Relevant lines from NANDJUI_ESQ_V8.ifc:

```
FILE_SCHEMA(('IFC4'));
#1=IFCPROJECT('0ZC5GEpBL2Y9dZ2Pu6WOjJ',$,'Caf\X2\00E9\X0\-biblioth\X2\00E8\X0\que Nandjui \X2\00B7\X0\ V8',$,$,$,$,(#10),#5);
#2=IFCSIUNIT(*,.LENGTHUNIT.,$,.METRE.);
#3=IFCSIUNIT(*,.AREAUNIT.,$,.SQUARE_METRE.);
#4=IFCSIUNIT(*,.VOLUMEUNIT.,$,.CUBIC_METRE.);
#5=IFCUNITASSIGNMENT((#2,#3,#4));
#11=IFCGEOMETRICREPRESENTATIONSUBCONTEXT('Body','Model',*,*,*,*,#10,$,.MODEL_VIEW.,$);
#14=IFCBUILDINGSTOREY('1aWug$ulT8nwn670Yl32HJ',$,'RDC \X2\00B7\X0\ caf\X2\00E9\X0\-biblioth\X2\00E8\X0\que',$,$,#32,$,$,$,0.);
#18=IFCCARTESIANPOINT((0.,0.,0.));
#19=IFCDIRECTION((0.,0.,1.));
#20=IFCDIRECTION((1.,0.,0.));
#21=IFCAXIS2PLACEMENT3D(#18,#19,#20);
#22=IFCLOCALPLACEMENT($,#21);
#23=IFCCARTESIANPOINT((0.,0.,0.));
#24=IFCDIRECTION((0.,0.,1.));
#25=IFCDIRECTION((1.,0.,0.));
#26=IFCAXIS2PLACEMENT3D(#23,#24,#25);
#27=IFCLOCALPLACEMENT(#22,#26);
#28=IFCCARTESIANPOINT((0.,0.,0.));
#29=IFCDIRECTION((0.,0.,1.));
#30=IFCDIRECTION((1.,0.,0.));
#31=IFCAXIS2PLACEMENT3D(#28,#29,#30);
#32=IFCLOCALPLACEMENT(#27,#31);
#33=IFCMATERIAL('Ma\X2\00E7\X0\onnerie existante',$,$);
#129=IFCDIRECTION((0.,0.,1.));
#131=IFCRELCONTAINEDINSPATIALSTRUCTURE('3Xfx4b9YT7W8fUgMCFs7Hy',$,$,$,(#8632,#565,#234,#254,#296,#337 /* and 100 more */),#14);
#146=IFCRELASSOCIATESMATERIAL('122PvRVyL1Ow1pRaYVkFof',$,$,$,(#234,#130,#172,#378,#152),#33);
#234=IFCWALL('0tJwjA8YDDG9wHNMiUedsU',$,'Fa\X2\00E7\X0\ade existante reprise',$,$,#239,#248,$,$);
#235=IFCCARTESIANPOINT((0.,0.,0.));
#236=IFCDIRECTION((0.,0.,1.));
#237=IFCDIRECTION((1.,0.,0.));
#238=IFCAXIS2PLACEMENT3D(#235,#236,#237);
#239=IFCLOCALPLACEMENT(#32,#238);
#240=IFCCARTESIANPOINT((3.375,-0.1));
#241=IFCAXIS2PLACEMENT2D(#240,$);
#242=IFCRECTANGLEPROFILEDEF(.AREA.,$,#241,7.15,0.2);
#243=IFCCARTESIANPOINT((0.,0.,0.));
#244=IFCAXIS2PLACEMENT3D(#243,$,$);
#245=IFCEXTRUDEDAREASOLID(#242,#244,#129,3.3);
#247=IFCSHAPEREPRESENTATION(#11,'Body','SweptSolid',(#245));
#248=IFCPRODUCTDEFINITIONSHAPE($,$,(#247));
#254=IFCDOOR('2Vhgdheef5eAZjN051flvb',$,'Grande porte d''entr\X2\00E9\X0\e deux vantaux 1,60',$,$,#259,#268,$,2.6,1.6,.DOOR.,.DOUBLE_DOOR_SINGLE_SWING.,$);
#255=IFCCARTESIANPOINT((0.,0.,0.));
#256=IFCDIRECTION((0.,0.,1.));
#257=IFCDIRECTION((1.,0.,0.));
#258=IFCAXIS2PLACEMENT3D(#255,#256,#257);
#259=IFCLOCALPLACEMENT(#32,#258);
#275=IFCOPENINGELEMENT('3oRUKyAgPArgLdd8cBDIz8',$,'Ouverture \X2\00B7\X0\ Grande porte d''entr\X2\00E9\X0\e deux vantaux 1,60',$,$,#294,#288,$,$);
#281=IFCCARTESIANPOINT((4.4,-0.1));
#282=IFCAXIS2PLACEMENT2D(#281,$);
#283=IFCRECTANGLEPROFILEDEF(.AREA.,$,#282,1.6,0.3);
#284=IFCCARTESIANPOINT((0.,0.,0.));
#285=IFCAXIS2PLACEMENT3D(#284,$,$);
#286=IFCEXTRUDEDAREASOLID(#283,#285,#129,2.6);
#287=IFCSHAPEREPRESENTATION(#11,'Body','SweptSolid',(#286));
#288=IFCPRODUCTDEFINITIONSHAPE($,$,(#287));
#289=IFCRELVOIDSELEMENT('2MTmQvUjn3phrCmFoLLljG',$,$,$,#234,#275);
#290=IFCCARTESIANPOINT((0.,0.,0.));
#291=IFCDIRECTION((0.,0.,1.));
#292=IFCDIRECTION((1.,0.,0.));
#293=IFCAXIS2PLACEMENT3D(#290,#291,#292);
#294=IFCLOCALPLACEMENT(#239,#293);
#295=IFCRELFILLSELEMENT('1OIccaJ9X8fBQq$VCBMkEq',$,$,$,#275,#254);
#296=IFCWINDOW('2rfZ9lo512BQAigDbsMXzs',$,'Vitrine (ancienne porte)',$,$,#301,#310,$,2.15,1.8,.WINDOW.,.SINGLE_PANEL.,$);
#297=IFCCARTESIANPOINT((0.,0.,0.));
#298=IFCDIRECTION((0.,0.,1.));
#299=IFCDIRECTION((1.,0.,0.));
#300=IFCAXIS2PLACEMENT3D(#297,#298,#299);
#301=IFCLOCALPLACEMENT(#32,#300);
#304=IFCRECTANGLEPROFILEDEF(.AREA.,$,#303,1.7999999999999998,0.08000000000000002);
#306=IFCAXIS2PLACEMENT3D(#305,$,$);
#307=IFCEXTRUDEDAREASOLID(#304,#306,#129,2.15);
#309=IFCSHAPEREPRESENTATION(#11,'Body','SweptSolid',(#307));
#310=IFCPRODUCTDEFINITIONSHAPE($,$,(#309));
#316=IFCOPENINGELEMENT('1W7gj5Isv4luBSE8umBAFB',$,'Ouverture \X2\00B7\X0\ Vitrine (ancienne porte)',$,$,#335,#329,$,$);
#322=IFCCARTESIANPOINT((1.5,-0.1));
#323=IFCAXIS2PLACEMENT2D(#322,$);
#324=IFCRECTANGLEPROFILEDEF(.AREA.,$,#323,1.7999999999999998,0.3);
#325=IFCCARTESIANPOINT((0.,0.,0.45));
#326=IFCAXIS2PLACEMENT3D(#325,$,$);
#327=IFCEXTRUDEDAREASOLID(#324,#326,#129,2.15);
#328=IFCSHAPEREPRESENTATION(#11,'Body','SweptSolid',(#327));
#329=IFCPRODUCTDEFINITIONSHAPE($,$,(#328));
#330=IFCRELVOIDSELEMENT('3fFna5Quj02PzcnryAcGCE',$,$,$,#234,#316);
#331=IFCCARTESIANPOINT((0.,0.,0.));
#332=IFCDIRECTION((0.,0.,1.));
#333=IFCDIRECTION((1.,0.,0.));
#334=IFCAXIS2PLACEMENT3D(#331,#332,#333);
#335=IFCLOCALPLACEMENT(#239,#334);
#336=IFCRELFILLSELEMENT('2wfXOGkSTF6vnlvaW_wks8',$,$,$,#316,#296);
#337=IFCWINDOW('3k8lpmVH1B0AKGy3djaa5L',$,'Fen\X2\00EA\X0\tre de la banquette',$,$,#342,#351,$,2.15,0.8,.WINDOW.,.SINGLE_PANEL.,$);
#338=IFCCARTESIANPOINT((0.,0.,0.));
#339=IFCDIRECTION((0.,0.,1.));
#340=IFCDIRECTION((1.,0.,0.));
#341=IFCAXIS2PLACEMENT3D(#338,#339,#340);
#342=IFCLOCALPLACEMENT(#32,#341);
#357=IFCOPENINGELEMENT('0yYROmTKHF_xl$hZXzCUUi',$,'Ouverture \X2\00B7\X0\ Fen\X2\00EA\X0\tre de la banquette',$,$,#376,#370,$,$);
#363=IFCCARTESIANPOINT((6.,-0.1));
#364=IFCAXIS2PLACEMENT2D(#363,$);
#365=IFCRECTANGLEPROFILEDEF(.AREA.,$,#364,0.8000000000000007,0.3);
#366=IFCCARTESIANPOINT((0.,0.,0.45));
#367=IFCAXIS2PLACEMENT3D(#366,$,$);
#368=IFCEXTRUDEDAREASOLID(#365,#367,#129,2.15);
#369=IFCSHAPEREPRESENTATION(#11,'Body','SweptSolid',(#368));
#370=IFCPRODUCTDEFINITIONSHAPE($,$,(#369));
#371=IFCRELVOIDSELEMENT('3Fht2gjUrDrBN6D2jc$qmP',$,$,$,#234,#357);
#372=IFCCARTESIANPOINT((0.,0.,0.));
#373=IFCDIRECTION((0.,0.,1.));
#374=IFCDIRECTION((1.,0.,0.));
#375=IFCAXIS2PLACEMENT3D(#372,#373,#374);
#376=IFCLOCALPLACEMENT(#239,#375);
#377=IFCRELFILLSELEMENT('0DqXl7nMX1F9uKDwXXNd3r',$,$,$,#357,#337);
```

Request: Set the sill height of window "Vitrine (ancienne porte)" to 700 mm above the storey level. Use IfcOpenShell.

```python
import numpy as np
import ifcopenshell
import ifcopenshell.api.geometry
import ifcopenshell.geom
import ifcopenshell.util.element
import ifcopenshell.util.placement
import ifcopenshell.util.shape
import ifcopenshell.util.unit

model = ifcopenshell.open("NANDJUI_ESQ_V8.ifc")
unit_scale = ifcopenshell.util.unit.calculate_unit_scale(model)

window = model.by_id(296)
opening = window.FillsVoids[0].RelatingOpeningElement
storey = ifcopenshell.util.element.get_container(window, ifc_class="IfcBuildingStorey")
level = ifcopenshell.util.placement.get_local_placement(storey.ObjectPlacement)[2, 3]

# The opening's origin need not be at the sill, so measure its lowest point.
shape = ifcopenshell.geom.create_shape(ifcopenshell.geom.settings(), opening)
bottom = ifcopenshell.util.shape.get_shape_bottom_elevation(shape, shape.geometry) / unit_scale
dz = level + 0.7 / unit_scale - bottom

shift = np.array([0.0, 0.0, dz])
# The window is not placed relative to its opening, so move both.
for product in (opening, window):
    matrix = ifcopenshell.util.placement.get_local_placement(product.ObjectPlacement)
    matrix[:3, 3] += shift
    ifcopenshell.api.geometry.edit_object_placement(model, product=product, matrix=matrix, is_si=False)

print(f"moved by {dz * unit_scale:+.3f} m")

model.write("NANDJUI_ESQ_V8_rev.ifc")
```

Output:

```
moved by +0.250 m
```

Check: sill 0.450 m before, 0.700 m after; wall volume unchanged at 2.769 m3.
